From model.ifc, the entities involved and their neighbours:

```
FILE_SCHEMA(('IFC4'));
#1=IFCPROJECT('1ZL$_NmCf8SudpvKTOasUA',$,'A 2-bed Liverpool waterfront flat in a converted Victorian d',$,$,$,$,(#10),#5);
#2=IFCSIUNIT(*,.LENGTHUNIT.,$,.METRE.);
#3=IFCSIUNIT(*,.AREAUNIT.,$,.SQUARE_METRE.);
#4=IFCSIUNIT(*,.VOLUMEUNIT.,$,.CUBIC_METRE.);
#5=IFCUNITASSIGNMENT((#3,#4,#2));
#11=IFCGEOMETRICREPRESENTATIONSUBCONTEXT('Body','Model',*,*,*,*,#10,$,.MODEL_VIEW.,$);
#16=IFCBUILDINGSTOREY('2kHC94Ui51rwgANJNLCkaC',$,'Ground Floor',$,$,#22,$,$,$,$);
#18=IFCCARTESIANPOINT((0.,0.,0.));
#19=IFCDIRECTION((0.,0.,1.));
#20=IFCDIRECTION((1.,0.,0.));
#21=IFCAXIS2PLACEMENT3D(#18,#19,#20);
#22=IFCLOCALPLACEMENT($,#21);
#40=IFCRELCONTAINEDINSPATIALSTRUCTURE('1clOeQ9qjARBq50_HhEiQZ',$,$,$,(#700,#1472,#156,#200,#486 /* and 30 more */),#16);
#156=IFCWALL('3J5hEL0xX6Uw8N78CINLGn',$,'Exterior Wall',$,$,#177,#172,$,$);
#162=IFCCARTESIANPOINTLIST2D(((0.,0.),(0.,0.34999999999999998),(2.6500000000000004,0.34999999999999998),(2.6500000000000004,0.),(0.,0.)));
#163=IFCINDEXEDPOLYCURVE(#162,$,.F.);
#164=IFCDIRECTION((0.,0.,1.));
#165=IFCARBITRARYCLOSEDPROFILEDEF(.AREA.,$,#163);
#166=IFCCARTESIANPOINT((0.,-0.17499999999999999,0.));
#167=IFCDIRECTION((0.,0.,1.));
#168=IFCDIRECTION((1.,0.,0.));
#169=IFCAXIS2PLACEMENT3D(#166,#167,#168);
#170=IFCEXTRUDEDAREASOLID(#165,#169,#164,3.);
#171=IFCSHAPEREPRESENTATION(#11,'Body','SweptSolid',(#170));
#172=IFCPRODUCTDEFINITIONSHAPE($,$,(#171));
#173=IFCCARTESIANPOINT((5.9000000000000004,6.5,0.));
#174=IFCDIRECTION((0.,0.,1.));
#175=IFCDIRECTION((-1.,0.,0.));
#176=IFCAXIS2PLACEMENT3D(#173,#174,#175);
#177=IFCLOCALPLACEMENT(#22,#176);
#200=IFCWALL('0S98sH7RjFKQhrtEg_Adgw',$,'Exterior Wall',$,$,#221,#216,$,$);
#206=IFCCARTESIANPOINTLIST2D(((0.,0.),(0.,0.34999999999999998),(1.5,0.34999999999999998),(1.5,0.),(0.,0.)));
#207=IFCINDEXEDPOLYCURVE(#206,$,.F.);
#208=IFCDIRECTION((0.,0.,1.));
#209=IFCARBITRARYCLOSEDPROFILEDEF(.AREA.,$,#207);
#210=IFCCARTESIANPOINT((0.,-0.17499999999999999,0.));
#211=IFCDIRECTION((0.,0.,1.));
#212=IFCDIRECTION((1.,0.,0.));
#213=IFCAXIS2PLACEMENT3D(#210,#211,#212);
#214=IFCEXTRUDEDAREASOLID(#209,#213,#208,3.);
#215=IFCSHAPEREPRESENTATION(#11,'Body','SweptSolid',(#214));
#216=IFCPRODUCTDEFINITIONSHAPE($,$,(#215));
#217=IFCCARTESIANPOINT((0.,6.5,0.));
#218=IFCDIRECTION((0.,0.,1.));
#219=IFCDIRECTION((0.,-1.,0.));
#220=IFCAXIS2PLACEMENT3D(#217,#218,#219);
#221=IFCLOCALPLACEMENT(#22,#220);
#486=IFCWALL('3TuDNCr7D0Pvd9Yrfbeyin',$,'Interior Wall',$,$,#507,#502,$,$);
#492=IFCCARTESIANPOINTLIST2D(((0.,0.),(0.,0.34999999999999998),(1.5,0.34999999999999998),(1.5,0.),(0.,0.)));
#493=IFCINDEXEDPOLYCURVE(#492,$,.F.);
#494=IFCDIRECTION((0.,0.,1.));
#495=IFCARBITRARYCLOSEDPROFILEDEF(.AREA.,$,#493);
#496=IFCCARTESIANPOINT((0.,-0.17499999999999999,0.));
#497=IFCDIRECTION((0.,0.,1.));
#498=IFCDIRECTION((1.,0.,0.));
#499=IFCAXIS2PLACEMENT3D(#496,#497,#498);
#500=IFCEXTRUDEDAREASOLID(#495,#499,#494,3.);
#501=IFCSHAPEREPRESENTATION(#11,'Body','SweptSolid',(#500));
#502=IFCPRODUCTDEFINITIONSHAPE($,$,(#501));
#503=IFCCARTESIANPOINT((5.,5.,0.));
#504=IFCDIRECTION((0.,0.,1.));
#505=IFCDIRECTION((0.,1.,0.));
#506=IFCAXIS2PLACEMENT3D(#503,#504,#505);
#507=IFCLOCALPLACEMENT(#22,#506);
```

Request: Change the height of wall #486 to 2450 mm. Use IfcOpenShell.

```python
import ifcopenshell
import ifcopenshell.geom
import ifcopenshell.util.representation
import ifcopenshell.util.shape

model = ifcopenshell.open("model.ifc")
settings = ifcopenshell.geom.settings()


def volume(element):
    """Net volume in cubic metres, openings subtracted."""
    shape = ifcopenshell.geom.create_shape(settings, element)
    return ifcopenshell.util.shape.get_volume(shape.geometry)


wall = model.by_id(486)
before = volume(wall)

body = ifcopenshell.util.representation.get_representation(wall, "Model", "Body")
solid = body.Items[0]
old_height = solid.Depth
solid.Depth = 2.45
after = volume(wall)

print(f"height {old_height:g} -> {solid.Depth:g}, volume {before:.3f} -> {after:.3f} m3")

model.write("model_edited.ifc")
```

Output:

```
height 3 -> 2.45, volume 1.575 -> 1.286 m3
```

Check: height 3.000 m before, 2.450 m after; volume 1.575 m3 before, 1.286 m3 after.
